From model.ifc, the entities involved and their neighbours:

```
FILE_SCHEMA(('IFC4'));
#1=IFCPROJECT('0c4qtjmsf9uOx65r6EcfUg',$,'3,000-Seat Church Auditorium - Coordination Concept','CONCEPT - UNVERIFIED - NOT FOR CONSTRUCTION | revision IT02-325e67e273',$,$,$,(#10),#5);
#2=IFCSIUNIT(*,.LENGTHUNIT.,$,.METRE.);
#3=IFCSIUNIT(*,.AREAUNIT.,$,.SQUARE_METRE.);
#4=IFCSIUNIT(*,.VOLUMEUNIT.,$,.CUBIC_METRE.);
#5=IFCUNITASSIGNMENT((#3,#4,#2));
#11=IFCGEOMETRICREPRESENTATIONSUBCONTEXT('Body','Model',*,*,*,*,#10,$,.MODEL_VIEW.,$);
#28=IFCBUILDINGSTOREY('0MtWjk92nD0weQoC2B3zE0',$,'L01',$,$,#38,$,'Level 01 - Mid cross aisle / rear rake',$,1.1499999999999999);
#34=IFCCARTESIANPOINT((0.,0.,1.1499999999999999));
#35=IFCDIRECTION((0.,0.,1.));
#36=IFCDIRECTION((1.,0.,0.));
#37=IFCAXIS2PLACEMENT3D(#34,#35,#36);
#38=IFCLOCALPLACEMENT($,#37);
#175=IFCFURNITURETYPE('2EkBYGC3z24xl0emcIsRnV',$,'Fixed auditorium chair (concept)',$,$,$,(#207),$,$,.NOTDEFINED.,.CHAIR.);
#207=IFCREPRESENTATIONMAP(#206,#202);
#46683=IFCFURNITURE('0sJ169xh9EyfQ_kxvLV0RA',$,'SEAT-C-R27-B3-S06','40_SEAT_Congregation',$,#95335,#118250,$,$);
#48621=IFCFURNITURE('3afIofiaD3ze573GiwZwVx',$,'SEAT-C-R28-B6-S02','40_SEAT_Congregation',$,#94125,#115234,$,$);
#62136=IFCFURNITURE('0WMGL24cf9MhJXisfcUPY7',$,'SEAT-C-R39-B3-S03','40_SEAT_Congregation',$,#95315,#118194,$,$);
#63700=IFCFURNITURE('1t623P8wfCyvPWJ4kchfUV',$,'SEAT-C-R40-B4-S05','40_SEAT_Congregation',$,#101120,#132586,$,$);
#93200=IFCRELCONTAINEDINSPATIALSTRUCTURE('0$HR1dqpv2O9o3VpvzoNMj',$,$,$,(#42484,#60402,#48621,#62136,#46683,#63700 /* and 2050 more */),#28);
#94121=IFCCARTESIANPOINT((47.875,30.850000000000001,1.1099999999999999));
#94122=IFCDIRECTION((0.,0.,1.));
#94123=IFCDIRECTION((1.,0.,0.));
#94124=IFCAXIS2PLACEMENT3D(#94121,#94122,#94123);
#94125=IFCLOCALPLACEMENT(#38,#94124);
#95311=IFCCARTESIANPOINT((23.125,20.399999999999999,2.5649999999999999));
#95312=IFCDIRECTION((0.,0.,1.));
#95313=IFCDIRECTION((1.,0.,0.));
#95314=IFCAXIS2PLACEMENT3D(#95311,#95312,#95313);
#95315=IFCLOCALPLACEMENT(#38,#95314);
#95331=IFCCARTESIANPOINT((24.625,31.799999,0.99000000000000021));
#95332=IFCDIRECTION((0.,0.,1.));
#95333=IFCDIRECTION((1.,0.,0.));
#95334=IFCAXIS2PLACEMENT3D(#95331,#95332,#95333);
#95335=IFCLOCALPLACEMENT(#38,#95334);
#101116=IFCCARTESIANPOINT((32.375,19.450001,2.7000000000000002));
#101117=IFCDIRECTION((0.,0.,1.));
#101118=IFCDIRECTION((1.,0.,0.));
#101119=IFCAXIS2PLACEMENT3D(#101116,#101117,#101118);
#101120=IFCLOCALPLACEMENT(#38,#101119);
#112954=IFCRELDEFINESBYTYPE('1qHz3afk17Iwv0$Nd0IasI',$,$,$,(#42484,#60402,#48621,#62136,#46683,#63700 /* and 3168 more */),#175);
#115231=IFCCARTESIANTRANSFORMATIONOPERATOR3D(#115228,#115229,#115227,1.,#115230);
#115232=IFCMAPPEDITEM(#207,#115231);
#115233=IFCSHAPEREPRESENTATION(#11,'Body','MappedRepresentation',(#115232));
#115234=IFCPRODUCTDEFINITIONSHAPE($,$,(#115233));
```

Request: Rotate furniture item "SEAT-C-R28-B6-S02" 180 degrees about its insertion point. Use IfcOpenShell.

```python
import ifcopenshell
import ifcopenshell.api.geometry
import ifcopenshell.util.placement

model = ifcopenshell.open("model.ifc")

item = model.by_guid("3afIofiaD3ze573GiwZwVx")
matrix = ifcopenshell.util.placement.get_local_placement(item.ObjectPlacement)
matrix = matrix @ ifcopenshell.util.placement.rotation(180, "Z")
ifcopenshell.api.geometry.edit_object_placement(model, product=item, matrix=matrix, is_si=False)

print(ifcopenshell.util.placement.get_local_placement(item.ObjectPlacement).round(3) + 0.0)

model.write("model_updated.ifc")
```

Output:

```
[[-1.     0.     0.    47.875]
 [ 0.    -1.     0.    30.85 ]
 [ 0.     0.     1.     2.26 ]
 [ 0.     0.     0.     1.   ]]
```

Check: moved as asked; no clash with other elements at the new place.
